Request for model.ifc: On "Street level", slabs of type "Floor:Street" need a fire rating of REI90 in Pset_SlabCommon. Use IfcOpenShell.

First a look at what the model holds.

```python
import ifcopenshell
import ifcopenshell.util.element

model = ifcopenshell.open("model.ifc")
print(model.schema)
storey = next(s for s in model.by_type("IfcBuildingStorey") if s.Name == "Street level")
slabs = [e for e in ifcopenshell.util.element.get_decomposition(storey) if e.is_a("IfcSlab")]
seen = {}
for e in slabs:
    element_type = ifcopenshell.util.element.get_type(e)
    key = (element_type.Name if element_type != e and element_type else None, ifcopenshell.util.element.get_pset(e, "Pset_SlabCommon", "FireRating"))
    seen[key] = seen.get(key, 0) + 1
for (name, value), count in sorted(seen.items(), key=str):
    print(count, "x", name, "|", value)
```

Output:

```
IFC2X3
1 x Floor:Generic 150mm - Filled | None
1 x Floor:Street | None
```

```python
import ifcopenshell
import ifcopenshell.api.pset
import ifcopenshell.util.element

model = ifcopenshell.open("model.ifc")

storey = next(s for s in model.by_type("IfcBuildingStorey") if s.Name == "Street level")
slabs = [e for e in ifcopenshell.util.element.get_decomposition(storey) if e.is_a("IfcSlab")]

count = 0
for e in slabs:
    element_type = ifcopenshell.util.element.get_type(e)
    if element_type in (None, e) or element_type.Name != "Floor:Street":
        continue
    # add_pset returns the element's existing set when there is one.
    pset = ifcopenshell.api.pset.add_pset(model, product=e, name="Pset_SlabCommon")
    ifcopenshell.api.pset.edit_pset(model, pset=pset, properties={"FireRating": "REI90"})
    count += 1

print(count, "slabs updated")

model.write("model_rev.ifc")
```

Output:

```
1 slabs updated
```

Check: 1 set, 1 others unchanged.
